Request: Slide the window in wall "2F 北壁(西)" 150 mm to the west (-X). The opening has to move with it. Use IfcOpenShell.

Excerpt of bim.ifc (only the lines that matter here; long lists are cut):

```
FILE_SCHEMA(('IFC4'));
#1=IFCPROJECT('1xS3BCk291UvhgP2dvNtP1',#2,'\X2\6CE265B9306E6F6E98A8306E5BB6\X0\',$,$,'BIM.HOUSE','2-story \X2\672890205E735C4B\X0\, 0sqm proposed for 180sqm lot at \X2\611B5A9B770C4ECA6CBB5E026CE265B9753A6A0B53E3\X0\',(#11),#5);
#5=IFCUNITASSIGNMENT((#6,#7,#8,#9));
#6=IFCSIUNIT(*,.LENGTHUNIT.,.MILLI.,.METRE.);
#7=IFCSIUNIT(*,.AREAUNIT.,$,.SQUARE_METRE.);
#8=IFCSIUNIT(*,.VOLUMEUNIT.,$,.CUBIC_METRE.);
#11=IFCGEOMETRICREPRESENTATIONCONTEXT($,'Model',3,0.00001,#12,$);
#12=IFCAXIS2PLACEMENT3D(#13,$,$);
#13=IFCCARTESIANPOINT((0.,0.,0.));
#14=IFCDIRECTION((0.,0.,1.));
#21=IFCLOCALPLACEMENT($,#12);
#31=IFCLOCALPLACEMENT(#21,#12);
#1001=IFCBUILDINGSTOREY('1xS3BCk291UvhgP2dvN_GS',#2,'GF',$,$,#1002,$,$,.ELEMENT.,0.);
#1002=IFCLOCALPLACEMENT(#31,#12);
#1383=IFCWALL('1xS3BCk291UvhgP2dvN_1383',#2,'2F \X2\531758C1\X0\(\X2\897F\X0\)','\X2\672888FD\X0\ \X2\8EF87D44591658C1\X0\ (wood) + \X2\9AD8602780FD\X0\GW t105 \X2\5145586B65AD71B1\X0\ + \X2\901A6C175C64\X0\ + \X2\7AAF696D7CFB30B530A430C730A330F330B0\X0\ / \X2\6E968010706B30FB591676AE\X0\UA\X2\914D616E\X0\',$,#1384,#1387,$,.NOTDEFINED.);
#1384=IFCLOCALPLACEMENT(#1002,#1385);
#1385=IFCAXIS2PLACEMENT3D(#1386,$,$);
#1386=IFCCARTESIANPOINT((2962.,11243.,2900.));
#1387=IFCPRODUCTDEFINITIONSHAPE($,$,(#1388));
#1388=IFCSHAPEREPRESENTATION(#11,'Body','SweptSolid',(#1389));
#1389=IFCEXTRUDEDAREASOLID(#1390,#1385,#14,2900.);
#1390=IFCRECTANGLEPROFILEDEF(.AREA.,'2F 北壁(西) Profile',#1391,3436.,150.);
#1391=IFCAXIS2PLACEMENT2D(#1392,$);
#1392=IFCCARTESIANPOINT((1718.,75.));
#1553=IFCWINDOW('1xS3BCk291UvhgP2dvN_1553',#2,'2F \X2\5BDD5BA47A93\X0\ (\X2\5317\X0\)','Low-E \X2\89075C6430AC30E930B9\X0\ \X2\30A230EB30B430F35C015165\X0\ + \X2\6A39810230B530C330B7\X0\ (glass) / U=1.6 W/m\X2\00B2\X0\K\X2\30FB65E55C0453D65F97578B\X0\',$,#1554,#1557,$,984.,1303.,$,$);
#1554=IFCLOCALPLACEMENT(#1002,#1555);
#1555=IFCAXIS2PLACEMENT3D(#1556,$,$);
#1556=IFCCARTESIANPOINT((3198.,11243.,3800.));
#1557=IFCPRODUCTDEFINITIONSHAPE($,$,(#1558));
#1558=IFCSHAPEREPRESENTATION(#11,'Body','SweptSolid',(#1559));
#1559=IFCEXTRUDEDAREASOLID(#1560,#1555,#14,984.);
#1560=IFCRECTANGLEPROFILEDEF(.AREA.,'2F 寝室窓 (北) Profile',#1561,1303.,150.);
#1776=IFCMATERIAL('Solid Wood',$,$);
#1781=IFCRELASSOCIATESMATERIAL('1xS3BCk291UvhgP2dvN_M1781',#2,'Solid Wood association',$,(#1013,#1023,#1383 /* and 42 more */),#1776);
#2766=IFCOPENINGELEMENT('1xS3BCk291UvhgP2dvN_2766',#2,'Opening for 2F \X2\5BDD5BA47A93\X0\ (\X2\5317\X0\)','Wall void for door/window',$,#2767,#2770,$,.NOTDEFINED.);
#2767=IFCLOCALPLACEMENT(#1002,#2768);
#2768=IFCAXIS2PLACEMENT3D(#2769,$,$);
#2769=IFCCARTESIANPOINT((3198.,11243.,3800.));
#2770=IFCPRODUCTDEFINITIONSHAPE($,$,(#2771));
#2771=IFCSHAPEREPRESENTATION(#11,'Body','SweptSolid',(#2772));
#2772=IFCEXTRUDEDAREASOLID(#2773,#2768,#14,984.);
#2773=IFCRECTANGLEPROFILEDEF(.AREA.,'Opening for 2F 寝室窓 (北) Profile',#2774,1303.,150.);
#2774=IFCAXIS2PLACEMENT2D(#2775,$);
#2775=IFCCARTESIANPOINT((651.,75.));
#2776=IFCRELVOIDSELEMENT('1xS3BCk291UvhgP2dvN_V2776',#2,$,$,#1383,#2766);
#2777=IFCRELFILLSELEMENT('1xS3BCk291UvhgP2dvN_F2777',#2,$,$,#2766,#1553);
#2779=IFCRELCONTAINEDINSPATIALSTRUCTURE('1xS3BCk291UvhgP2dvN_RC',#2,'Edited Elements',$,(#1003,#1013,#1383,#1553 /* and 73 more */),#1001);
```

```python
import ifcopenshell
import ifcopenshell.api.geometry
import ifcopenshell.util.placement
import ifcopenshell.util.unit

model = ifcopenshell.open("bim.ifc")
unit_scale = ifcopenshell.util.unit.calculate_unit_scale(model)

window = model.by_id(1553)
opening = window.FillsVoids[0].RelatingOpeningElement
wall = opening.VoidsElements[0].RelatingBuildingElement

wall_matrix = ifcopenshell.util.placement.get_local_placement(wall.ObjectPlacement)
shift = wall_matrix[:3, 0] * -0.15 / unit_scale
before = ifcopenshell.util.placement.get_local_placement(window.ObjectPlacement)[:3, 3].copy()

# The window is not placed relative to its opening, so move both.
for product in (opening, window):
    matrix = ifcopenshell.util.placement.get_local_placement(product.ObjectPlacement)
    matrix[:3, 3] += shift
    ifcopenshell.api.geometry.edit_object_placement(model, product=product, matrix=matrix, is_si=False)

after = ifcopenshell.util.placement.get_local_placement(window.ObjectPlacement)[:3, 3]
print("window moved by", (after - before).round(3) + 0.0)

model.write("bim_rev.ifc")
```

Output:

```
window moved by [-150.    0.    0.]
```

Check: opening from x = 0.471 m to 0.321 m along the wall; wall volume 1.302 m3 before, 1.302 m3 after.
